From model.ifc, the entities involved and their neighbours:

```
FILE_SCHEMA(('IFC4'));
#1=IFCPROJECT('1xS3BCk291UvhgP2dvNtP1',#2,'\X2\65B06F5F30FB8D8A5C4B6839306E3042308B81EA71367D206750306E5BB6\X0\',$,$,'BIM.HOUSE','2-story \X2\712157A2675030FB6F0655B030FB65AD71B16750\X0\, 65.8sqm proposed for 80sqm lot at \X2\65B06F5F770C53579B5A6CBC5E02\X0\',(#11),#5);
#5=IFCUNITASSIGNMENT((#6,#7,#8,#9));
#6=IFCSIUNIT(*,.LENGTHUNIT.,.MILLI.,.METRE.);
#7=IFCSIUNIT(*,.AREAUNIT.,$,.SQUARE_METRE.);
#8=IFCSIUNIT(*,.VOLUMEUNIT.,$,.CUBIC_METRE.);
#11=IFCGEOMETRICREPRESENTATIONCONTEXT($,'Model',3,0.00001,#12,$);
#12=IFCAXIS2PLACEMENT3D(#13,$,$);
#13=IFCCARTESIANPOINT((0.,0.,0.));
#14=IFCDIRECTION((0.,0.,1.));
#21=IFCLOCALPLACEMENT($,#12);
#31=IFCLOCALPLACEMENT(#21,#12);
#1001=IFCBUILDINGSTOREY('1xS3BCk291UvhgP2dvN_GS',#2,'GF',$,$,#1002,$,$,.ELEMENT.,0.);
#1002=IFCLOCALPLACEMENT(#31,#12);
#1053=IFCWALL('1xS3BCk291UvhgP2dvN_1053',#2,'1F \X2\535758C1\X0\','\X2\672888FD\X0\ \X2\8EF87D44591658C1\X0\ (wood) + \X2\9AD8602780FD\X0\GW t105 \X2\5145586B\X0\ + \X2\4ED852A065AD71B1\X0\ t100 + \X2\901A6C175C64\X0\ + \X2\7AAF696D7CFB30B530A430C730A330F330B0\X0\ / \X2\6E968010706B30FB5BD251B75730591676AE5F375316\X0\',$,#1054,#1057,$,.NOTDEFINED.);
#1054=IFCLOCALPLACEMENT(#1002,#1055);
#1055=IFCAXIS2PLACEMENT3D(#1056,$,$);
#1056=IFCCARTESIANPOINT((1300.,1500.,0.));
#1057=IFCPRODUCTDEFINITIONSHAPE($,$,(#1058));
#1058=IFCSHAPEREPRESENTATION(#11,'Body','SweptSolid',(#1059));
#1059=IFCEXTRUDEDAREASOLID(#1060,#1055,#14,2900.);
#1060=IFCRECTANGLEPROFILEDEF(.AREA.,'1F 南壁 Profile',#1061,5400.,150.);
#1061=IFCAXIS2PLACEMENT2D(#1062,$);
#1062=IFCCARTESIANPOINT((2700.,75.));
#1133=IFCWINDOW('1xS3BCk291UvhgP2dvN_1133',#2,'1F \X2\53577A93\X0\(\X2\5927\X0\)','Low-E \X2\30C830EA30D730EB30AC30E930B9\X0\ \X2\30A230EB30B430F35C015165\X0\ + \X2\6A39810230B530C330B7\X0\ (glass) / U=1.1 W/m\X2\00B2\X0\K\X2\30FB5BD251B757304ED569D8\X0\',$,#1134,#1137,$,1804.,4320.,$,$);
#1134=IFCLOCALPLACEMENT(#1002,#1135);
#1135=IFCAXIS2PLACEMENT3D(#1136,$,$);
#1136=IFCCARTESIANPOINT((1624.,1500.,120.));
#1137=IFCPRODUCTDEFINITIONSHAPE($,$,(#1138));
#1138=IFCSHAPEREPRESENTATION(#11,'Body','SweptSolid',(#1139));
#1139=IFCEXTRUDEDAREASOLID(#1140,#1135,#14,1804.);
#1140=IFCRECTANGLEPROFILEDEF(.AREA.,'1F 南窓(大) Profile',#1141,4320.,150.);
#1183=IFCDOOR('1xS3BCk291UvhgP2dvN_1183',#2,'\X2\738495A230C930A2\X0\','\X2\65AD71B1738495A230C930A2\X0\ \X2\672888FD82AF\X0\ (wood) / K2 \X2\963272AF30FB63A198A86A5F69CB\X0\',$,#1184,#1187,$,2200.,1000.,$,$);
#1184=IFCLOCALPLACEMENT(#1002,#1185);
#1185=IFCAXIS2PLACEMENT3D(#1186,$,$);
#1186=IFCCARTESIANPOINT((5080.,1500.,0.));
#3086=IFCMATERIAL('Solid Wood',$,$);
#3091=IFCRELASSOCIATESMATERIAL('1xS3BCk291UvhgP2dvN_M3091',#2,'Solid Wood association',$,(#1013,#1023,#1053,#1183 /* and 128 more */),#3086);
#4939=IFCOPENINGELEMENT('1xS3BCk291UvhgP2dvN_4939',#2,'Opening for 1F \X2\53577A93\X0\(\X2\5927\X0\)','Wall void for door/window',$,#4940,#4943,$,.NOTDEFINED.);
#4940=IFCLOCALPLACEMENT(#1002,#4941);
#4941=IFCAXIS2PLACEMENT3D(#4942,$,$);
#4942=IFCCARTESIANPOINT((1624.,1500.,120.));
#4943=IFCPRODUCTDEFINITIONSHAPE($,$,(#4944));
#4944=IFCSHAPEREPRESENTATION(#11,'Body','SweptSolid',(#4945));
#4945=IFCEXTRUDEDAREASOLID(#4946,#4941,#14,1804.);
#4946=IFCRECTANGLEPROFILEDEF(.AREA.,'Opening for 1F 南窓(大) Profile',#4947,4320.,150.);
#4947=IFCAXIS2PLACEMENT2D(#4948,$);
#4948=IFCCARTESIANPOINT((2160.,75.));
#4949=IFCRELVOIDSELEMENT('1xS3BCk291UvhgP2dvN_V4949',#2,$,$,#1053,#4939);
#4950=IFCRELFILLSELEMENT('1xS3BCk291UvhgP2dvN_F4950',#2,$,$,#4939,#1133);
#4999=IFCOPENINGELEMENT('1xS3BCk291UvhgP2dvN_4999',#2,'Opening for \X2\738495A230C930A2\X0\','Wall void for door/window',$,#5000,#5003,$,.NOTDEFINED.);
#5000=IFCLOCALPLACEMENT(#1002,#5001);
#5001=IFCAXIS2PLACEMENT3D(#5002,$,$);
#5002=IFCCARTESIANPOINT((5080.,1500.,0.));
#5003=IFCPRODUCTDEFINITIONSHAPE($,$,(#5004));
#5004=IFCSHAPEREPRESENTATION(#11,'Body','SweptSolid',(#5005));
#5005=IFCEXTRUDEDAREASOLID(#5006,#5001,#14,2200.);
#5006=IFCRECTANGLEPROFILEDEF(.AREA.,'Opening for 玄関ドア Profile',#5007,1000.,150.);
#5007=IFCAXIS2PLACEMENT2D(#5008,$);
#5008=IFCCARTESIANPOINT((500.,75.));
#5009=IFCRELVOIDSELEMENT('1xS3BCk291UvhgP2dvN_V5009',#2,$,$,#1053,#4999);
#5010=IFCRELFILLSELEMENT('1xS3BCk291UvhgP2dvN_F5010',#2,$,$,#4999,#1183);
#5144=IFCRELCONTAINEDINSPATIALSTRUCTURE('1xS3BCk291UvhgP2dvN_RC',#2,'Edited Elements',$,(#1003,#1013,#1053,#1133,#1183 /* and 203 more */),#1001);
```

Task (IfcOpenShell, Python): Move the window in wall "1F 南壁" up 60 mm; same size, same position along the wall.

```python
import numpy as np
import ifcopenshell
import ifcopenshell.api.geometry
import ifcopenshell.util.placement
import ifcopenshell.util.unit

model = ifcopenshell.open("model.ifc")
unit_scale = ifcopenshell.util.unit.calculate_unit_scale(model)

window = model.by_id(1133)
opening = window.FillsVoids[0].RelatingOpeningElement
dz = 60.0

shift = np.array([0.0, 0.0, dz])
# The window is not placed relative to its opening, so move both.
for product in (opening, window):
    matrix = ifcopenshell.util.placement.get_local_placement(product.ObjectPlacement)
    matrix[:3, 3] += shift
    ifcopenshell.api.geometry.edit_object_placement(model, product=product, matrix=matrix, is_si=False)

print(f"moved by {dz * unit_scale:+.3f} m")

model.write("model-out.ifc")
```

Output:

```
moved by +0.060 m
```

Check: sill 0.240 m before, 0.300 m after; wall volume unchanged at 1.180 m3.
